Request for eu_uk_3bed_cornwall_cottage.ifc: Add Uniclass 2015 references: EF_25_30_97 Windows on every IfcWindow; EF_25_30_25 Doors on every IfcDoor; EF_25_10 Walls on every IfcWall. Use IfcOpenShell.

First a look at what the model holds.

```python
import ifcopenshell

model = ifcopenshell.open("eu_uk_3bed_cornwall_cottage.ifc")
print(model.schema)
print("classifications:", [c.Name for c in model.by_type("IfcClassification")])
for ifc_class in ("IfcDoor", "IfcRoof", "IfcStair", "IfcWall", "IfcWindow"):
    print(ifc_class, len(model.by_type(ifc_class)))
```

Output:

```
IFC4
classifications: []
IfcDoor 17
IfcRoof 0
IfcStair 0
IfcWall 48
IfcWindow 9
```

```python
import ifcopenshell
import ifcopenshell.api.classification

model = ifcopenshell.open("eu_uk_3bed_cornwall_cottage.ifc")

system = ifcopenshell.api.classification.add_classification(model, classification="Uniclass 2015")

codes = {
    "IfcWindow": ("EF_25_30_97", "Windows"),
    "IfcDoor": ("EF_25_30_25", "Doors"),
    "IfcWall": ("EF_25_10", "Walls"),
}
for ifc_class, (code, name) in codes.items():
    products = model.by_type(ifc_class)
    ifcopenshell.api.classification.add_reference(
        model, products=products, classification=system, identification=code, name=name
    )
    print(code, len(products))

model.write("eu_uk_3bed_cornwall_cottage_rev.ifc")
```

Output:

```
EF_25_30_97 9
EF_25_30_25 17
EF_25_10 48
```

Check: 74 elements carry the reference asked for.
